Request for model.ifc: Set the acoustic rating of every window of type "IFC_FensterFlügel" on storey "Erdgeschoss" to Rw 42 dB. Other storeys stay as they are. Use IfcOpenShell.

First a look at what the model holds.

```python
import ifcopenshell
import ifcopenshell.util.element

model = ifcopenshell.open("model.ifc")
print(model.schema)
storey = next(s for s in model.by_type("IfcBuildingStorey") if s.Name == "Erdgeschoss")
windows = [e for e in ifcopenshell.util.element.get_decomposition(storey) if e.is_a("IfcWindow")]
seen = {}
for e in windows:
    element_type = ifcopenshell.util.element.get_type(e)
    key = (element_type.Name if element_type != e and element_type else None, ifcopenshell.util.element.get_pset(e, "Pset_WindowCommon", "AcousticRating"))
    seen[key] = seen.get(key, 0) + 1
for (name, value), count in sorted(seen.items(), key=str):
    print(count, "x", name, "|", value)
```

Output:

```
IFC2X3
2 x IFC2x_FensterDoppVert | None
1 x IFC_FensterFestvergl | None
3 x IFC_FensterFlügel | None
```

```python
import ifcopenshell
import ifcopenshell.api.pset
import ifcopenshell.util.element

model = ifcopenshell.open("model.ifc")

storey = next(s for s in model.by_type("IfcBuildingStorey") if s.Name == "Erdgeschoss")
windows = [e for e in ifcopenshell.util.element.get_decomposition(storey) if e.is_a("IfcWindow")]

count = 0
for e in windows:
    element_type = ifcopenshell.util.element.get_type(e)
    if element_type in (None, e) or element_type.Name != "IFC_FensterFlügel":
        continue
    # add_pset returns the element's existing set when there is one.
    pset = ifcopenshell.api.pset.add_pset(model, product=e, name="Pset_WindowCommon")
    ifcopenshell.api.pset.edit_pset(model, pset=pset, properties={"AcousticRating": "Rw 42 dB"})
    count += 1

print(count, "windows updated")

model.write("model_updated.ifc")
```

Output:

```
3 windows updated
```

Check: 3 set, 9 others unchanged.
